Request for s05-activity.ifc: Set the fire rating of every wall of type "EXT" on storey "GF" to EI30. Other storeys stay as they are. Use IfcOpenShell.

First a look at what the model holds.

```python
import ifcopenshell
import ifcopenshell.util.element

model = ifcopenshell.open("s05-activity.ifc")
print(model.schema)
storey = next(s for s in model.by_type("IfcBuildingStorey") if s.Name == "GF")
walls = [e for e in ifcopenshell.util.element.get_decomposition(storey) if e.is_a("IfcWall")]
seen = {}
for e in walls:
    element_type = ifcopenshell.util.element.get_type(e)
    key = (element_type.Name if element_type != e and element_type else None, ifcopenshell.util.element.get_pset(e, "Pset_WallCommon", "FireRating"))
    seen[key] = seen.get(key, 0) + 1
for (name, value), count in sorted(seen.items(), key=str):
    print(count, "x", name, "|", value)
```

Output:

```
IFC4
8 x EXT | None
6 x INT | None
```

```python
import ifcopenshell
import ifcopenshell.api.pset
import ifcopenshell.util.element

model = ifcopenshell.open("s05-activity.ifc")

storey = next(s for s in model.by_type("IfcBuildingStorey") if s.Name == "GF")
walls = [e for e in ifcopenshell.util.element.get_decomposition(storey) if e.is_a("IfcWall")]

count = 0
for e in walls:
    element_type = ifcopenshell.util.element.get_type(e)
    if element_type in (None, e) or element_type.Name != "EXT":
        continue
    # add_pset returns the element's existing set when there is one.
    pset = ifcopenshell.api.pset.add_pset(model, product=e, name="Pset_WallCommon")
    ifcopenshell.api.pset.edit_pset(model, pset=pset, properties={"FireRating": "EI30"})
    count += 1

print(count, "walls updated")

model.write("s05-activity_edited.ifc")
```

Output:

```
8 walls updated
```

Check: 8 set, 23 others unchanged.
